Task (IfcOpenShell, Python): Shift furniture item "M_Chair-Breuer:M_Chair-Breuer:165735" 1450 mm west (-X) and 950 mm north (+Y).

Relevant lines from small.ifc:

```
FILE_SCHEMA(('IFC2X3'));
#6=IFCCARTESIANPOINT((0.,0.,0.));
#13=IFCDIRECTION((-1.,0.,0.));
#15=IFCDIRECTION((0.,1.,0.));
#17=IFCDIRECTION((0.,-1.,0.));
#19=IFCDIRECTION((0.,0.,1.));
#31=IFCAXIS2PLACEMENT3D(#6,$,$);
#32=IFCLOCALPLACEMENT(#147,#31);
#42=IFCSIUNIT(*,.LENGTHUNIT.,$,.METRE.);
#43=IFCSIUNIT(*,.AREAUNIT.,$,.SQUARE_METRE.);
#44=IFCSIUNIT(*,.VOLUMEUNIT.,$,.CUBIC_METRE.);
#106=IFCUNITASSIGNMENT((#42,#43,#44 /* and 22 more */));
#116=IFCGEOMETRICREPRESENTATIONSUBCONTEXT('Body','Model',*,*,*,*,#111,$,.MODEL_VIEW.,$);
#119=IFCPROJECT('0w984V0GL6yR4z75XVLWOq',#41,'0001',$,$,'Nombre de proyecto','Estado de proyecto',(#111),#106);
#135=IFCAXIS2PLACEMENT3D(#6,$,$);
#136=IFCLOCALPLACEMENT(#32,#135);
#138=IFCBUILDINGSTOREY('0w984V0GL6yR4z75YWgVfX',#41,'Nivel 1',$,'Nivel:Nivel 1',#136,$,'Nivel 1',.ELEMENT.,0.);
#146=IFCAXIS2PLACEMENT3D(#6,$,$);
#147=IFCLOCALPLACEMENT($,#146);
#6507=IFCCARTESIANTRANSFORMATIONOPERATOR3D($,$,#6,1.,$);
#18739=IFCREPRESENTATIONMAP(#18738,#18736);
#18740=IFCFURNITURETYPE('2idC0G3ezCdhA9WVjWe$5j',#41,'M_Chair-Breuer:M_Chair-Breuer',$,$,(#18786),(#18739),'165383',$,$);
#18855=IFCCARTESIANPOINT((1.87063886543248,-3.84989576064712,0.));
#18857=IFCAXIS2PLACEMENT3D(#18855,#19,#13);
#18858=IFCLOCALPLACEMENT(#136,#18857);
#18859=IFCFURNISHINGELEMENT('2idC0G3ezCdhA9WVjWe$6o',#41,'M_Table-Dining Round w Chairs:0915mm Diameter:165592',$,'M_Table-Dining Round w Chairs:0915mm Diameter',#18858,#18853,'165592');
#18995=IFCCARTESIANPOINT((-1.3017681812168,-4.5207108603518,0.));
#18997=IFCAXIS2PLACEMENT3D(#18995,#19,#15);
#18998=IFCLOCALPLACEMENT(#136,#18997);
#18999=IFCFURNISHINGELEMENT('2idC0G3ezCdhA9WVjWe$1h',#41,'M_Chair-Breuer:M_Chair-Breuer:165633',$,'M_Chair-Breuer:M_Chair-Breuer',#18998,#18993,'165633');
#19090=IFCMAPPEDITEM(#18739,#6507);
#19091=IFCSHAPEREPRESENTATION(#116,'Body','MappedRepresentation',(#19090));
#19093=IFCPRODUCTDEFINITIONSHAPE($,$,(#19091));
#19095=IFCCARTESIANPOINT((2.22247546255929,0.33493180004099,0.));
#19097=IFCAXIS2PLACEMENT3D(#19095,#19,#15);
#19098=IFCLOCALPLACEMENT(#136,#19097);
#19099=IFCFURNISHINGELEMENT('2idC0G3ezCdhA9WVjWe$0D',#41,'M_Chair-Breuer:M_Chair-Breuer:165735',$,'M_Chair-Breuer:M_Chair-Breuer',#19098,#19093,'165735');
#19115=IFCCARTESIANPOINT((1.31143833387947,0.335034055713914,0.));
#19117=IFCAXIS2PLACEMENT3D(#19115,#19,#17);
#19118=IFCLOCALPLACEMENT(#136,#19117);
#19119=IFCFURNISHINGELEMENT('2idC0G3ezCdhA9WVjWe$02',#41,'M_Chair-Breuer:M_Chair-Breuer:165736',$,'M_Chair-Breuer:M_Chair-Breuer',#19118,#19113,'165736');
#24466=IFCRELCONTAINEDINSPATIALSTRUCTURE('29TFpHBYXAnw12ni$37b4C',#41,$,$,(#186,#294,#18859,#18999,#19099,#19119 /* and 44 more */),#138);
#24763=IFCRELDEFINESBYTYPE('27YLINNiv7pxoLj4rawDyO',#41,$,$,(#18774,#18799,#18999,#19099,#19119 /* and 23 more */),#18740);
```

```python
import ifcopenshell
import ifcopenshell.api.geometry
import ifcopenshell.util.placement
import ifcopenshell.util.unit

model = ifcopenshell.open("small.ifc")
unit_scale = ifcopenshell.util.unit.calculate_unit_scale(model)

item = model.by_id(19099)
matrix = ifcopenshell.util.placement.get_local_placement(item.ObjectPlacement)
matrix[0, 3] -= 1.45 / unit_scale
matrix[1, 3] += 0.95 / unit_scale
ifcopenshell.api.geometry.edit_object_placement(model, product=item, matrix=matrix, is_si=False)

print(ifcopenshell.util.placement.get_local_placement(item.ObjectPlacement).round(3) + 0.0)

model.write("small_rev.ifc")
```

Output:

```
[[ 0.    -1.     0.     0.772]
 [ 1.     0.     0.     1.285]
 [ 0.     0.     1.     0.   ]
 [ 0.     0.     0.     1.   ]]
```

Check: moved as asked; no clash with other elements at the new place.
